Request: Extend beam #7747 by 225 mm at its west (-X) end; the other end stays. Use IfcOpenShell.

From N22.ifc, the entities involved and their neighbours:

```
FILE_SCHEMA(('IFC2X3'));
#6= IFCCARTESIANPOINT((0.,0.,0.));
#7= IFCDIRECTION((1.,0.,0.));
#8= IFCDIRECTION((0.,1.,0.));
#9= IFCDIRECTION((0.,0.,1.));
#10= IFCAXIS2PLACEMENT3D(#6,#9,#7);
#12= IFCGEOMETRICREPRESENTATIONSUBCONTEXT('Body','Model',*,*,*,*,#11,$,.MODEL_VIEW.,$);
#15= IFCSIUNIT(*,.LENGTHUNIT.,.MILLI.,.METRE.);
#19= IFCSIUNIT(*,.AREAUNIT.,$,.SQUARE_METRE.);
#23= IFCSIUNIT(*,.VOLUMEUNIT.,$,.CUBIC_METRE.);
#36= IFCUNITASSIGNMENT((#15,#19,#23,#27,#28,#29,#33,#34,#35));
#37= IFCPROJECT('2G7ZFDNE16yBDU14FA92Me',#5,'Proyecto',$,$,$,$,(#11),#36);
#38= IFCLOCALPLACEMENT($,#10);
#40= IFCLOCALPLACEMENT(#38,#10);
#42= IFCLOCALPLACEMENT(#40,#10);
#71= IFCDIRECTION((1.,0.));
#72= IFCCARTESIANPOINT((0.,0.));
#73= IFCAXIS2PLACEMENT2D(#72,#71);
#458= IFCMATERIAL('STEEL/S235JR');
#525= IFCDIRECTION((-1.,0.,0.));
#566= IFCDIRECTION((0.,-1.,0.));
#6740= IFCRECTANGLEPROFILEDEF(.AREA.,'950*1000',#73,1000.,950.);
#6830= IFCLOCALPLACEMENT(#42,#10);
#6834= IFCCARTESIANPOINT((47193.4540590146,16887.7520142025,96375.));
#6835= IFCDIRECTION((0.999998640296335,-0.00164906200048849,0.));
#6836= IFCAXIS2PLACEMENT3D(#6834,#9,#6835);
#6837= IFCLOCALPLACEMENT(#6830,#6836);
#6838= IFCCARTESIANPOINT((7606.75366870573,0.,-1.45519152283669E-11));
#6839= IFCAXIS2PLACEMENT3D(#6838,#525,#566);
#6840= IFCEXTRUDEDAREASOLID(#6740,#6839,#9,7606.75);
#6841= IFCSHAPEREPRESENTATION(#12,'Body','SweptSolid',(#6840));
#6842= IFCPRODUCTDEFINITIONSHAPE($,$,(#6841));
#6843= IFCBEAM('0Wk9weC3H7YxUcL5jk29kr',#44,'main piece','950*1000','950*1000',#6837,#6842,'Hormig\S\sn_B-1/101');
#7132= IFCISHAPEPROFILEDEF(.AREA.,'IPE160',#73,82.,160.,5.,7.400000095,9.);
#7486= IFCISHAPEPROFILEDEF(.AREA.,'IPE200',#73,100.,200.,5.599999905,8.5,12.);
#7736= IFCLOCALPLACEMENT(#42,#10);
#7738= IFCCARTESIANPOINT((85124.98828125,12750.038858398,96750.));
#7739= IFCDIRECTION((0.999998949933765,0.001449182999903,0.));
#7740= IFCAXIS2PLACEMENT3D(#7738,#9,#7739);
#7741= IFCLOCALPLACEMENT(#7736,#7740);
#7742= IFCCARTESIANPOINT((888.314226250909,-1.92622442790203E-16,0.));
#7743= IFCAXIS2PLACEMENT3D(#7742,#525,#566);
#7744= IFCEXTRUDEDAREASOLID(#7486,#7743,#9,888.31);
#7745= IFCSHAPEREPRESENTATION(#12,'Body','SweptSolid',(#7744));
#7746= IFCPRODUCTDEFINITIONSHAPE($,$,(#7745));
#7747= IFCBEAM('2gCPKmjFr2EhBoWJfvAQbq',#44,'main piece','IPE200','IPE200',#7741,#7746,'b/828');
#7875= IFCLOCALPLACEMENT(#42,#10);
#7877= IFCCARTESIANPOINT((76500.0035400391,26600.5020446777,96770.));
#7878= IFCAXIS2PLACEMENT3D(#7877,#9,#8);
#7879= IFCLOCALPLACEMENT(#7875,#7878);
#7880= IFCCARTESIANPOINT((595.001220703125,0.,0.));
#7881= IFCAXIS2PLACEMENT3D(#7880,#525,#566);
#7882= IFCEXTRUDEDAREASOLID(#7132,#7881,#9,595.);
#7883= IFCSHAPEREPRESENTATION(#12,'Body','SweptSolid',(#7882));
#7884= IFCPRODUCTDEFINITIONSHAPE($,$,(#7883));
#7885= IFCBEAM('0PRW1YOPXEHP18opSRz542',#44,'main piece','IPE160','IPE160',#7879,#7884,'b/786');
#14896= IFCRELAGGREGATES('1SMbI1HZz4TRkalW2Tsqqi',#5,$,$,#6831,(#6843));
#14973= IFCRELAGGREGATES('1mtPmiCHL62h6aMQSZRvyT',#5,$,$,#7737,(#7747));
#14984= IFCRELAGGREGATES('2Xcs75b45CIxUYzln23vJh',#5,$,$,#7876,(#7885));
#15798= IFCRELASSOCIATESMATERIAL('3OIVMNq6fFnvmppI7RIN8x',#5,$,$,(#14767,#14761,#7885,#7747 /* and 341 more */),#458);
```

```python
import ifcopenshell
import ifcopenshell.util.representation
import ifcopenshell.util.unit

model = ifcopenshell.open("N22.ifc")
unit_scale = ifcopenshell.util.unit.calculate_unit_scale(model)

member = model.by_id(7747)
change = 0.225 / unit_scale

# The extrusion runs towards the end named, so only its depth changes.
body = ifcopenshell.util.representation.get_representation(member, "Model", "Body")
solid = body.Items[0]
old_length = solid.Depth
solid.Depth += change

print(f"length {old_length:g} -> {solid.Depth:g}")

model.write("N22_updated.ifc")
```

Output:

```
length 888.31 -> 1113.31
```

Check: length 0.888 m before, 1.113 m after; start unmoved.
